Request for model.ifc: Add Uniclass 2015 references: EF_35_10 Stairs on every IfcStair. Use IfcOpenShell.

First a look at what the model holds.

```python
import ifcopenshell

model = ifcopenshell.open("model.ifc")
print(model.schema)
print("classifications:", [c.Name for c in model.by_type("IfcClassification")])
for ifc_class in ("IfcDoor", "IfcRoof", "IfcStair", "IfcWall", "IfcWindow"):
    print(ifc_class, len(model.by_type(ifc_class)))
```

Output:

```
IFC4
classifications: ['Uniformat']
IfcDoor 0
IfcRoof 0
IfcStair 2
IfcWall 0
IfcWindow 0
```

```python
import ifcopenshell
import ifcopenshell.api.classification

model = ifcopenshell.open("model.ifc")

system = ifcopenshell.api.classification.add_classification(model, classification="Uniclass 2015")

codes = {
    "IfcStair": ("EF_35_10", "Stairs"),
}
for ifc_class, (code, name) in codes.items():
    products = model.by_type(ifc_class)
    ifcopenshell.api.classification.add_reference(
        model, products=products, classification=system, identification=code, name=name
    )
    print(code, len(products))

model.write("model_edited.ifc")
```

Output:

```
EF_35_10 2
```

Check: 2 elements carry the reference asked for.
